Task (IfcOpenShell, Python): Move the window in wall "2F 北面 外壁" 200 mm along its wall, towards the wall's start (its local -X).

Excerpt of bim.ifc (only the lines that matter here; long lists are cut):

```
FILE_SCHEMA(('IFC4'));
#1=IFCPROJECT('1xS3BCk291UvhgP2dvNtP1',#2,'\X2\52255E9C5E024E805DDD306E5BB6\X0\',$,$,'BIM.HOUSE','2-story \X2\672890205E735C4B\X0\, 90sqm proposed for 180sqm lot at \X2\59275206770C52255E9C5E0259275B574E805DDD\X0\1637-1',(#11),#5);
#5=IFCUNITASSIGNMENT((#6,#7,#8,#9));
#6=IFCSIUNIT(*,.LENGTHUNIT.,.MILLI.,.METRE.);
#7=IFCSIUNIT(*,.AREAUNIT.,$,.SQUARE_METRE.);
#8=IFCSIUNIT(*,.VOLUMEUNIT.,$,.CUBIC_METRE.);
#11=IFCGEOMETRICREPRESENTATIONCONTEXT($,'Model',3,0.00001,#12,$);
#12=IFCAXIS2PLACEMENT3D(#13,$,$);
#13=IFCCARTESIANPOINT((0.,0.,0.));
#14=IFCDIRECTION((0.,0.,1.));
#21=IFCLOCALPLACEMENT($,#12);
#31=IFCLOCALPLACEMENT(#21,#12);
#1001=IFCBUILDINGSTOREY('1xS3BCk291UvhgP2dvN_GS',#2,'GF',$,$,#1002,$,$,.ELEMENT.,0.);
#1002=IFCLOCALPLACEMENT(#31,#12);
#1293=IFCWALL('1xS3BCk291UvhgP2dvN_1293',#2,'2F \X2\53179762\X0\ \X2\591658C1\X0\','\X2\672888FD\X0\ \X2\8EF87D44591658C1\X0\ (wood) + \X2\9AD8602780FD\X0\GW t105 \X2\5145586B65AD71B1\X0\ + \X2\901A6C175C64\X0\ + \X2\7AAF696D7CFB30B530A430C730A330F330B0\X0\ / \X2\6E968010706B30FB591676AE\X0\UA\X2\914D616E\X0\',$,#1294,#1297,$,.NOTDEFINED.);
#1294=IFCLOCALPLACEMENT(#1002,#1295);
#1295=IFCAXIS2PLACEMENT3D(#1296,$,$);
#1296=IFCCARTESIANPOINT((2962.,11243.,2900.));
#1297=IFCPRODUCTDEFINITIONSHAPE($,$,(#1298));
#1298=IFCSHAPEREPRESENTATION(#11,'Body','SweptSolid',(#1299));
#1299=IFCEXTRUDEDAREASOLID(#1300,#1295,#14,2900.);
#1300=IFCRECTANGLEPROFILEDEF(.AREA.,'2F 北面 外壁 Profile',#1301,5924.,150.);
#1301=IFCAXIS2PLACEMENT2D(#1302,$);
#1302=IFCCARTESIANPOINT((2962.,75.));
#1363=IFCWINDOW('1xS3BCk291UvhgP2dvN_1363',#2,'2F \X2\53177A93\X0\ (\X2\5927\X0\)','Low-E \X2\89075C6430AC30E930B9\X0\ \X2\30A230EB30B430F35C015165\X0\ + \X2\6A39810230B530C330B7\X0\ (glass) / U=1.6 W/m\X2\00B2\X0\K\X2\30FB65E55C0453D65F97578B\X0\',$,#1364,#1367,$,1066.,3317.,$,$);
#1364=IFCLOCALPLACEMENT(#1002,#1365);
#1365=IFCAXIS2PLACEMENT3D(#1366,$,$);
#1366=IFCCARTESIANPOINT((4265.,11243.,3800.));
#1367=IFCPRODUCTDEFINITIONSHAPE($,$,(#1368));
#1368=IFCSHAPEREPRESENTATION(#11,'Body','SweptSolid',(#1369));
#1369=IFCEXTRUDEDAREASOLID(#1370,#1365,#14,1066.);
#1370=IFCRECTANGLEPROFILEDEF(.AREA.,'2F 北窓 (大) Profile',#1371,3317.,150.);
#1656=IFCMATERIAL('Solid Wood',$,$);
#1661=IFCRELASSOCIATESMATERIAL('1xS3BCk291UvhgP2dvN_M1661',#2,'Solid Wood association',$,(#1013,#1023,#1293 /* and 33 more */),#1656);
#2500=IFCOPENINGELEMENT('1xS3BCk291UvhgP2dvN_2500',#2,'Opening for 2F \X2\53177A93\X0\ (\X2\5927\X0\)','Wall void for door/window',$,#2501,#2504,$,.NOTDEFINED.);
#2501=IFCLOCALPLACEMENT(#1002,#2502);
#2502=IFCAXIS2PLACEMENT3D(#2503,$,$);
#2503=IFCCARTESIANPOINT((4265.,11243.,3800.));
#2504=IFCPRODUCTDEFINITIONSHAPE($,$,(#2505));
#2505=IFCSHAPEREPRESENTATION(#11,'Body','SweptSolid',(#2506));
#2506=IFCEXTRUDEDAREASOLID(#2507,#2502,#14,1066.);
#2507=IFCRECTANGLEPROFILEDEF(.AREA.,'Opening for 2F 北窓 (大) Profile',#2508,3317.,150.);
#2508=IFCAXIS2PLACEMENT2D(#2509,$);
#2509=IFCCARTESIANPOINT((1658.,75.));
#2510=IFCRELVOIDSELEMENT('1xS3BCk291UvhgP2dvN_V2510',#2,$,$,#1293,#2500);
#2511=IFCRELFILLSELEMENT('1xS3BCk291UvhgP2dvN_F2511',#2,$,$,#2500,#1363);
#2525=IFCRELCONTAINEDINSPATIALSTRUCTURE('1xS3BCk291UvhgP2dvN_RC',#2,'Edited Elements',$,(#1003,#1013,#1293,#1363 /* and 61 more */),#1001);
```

```python
import ifcopenshell
import ifcopenshell.api.geometry
import ifcopenshell.util.placement

model = ifcopenshell.open("bim.ifc")

window = model.by_guid("1xS3BCk291UvhgP2dvN_1363")
opening = window.FillsVoids[0].RelatingOpeningElement
wall = opening.VoidsElements[0].RelatingBuildingElement

wall_matrix = ifcopenshell.util.placement.get_local_placement(wall.ObjectPlacement)
shift = wall_matrix[:3, 0] * -200.0
before = ifcopenshell.util.placement.get_local_placement(window.ObjectPlacement)[:3, 3].copy()

# The window is not placed relative to its opening, so move both.
for product in (opening, window):
    matrix = ifcopenshell.util.placement.get_local_placement(product.ObjectPlacement)
    matrix[:3, 3] += shift
    ifcopenshell.api.geometry.edit_object_placement(model, product=product, matrix=matrix, is_si=False)

after = ifcopenshell.util.placement.get_local_placement(window.ObjectPlacement)[:3, 3]
print("window moved by", (after - before).round(3) + 0.0)

model.write("bim_v2.ifc")
```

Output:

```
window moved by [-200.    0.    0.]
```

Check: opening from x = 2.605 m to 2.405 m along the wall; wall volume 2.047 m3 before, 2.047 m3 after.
